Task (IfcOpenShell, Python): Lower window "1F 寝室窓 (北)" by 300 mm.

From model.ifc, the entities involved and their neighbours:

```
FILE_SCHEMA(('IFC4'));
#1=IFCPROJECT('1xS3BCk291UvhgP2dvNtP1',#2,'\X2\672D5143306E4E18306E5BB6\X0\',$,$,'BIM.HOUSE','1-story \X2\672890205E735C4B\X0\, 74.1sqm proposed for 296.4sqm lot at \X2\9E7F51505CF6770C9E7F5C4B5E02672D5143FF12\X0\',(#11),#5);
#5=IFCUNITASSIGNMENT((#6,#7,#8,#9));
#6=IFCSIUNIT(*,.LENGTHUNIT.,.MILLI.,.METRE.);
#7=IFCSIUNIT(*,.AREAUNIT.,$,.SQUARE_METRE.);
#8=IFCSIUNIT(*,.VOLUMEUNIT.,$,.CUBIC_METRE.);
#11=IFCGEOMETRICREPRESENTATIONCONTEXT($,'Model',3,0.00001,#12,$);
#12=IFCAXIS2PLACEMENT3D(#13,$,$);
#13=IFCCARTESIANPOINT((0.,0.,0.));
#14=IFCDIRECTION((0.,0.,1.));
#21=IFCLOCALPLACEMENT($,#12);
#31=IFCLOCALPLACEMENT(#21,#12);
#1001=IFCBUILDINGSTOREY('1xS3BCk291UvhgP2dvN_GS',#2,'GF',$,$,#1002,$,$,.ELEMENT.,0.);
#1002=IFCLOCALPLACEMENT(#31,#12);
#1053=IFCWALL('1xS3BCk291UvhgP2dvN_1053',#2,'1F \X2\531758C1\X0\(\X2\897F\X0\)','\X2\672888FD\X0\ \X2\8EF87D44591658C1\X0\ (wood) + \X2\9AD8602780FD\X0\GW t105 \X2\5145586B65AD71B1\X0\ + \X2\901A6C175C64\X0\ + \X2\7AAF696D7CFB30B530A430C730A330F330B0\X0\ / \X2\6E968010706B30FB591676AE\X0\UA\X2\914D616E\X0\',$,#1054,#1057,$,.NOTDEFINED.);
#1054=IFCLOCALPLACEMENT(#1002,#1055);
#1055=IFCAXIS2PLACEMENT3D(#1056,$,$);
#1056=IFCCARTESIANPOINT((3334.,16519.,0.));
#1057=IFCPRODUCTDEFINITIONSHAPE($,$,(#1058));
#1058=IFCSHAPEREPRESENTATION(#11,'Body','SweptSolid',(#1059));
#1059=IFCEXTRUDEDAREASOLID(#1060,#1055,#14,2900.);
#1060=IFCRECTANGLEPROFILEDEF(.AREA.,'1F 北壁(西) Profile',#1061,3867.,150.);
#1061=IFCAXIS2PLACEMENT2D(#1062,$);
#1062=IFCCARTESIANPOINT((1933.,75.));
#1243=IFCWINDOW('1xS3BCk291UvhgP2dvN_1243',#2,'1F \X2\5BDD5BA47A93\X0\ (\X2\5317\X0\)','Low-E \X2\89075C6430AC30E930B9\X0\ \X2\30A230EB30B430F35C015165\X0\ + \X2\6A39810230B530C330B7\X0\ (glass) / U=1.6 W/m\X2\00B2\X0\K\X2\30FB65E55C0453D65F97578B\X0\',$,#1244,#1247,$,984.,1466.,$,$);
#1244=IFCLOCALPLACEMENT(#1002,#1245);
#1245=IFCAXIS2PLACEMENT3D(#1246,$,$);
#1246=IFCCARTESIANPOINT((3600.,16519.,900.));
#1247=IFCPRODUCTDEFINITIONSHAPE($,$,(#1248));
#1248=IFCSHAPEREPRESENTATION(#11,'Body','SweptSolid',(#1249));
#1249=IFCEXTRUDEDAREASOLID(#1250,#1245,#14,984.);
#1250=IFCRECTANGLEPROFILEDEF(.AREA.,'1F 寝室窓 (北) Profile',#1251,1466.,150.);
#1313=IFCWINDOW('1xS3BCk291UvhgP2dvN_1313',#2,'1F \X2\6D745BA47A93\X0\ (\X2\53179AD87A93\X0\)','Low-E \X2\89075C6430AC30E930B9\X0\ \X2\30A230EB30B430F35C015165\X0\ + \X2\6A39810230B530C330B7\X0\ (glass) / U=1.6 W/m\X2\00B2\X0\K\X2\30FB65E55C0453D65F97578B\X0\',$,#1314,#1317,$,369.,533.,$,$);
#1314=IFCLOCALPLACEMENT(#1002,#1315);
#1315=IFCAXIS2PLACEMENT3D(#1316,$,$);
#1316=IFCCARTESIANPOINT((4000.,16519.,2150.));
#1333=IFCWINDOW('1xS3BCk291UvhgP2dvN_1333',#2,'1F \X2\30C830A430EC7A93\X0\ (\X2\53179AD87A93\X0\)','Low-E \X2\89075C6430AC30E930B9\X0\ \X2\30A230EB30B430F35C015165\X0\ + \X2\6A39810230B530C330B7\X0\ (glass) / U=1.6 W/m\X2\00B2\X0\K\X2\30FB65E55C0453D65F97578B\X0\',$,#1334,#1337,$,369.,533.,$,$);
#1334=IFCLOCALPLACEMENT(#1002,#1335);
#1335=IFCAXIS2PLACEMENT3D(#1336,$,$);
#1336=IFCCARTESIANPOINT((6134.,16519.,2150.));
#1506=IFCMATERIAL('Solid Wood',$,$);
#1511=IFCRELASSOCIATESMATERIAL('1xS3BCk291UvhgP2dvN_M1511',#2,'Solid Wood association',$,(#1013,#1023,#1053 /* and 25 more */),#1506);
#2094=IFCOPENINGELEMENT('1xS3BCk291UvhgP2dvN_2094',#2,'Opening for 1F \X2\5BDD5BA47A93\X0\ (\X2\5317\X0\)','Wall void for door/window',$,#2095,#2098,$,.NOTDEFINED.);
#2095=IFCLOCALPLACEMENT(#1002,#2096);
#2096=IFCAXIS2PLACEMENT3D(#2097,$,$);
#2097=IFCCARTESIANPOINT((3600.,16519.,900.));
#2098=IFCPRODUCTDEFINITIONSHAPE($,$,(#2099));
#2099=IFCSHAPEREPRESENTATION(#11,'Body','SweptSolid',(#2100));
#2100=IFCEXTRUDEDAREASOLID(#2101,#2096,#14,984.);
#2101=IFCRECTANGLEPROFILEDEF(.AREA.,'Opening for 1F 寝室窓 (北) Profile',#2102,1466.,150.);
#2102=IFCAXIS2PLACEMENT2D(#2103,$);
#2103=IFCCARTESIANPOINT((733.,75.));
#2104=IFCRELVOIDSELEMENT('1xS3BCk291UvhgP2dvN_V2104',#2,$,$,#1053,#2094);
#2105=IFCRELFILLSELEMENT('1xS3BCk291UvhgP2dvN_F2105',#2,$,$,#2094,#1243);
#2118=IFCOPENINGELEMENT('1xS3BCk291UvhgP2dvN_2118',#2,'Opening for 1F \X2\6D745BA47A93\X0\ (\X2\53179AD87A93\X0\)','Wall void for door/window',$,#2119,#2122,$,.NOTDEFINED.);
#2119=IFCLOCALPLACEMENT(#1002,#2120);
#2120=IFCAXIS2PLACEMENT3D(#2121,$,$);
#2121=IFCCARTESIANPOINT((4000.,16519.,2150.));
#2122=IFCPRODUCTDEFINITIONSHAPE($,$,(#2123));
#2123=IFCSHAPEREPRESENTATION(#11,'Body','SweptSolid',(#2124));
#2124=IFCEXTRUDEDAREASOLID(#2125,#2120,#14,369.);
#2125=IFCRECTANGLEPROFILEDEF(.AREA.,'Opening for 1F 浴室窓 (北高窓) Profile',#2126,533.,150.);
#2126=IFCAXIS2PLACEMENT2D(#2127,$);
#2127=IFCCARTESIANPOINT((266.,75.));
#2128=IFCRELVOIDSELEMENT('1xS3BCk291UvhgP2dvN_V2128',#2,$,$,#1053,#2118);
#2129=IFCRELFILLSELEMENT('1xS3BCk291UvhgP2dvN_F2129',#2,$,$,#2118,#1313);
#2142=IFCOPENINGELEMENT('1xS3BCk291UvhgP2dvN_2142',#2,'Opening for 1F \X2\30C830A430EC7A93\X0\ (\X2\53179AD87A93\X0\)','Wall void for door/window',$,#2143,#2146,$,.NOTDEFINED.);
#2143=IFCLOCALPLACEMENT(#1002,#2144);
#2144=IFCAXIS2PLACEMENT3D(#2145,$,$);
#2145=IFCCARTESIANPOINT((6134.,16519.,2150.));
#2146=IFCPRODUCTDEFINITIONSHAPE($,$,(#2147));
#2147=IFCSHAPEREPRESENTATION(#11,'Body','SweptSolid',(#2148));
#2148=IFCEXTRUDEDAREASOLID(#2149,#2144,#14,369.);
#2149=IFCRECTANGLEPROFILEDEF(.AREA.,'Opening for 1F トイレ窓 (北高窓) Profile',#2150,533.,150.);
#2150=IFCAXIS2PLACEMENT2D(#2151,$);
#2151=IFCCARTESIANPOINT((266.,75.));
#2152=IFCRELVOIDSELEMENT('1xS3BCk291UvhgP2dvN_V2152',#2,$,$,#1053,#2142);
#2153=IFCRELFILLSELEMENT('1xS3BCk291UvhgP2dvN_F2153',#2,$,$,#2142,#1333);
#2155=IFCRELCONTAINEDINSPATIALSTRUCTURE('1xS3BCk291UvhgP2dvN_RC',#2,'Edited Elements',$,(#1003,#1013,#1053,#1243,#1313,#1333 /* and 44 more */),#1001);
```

```python
import numpy as np
import ifcopenshell
import ifcopenshell.api.geometry
import ifcopenshell.util.placement
import ifcopenshell.util.unit

model = ifcopenshell.open("model.ifc")
unit_scale = ifcopenshell.util.unit.calculate_unit_scale(model)

window = model.by_guid("1xS3BCk291UvhgP2dvN_1243")
opening = window.FillsVoids[0].RelatingOpeningElement
dz = -0.3 / unit_scale

shift = np.array([0.0, 0.0, dz])
# The window is not placed relative to its opening, so move both.
for product in (opening, window):
    matrix = ifcopenshell.util.placement.get_local_placement(product.ObjectPlacement)
    matrix[:3, 3] += shift
    ifcopenshell.api.geometry.edit_object_placement(model, product=product, matrix=matrix, is_si=False)

print(f"moved by {dz * unit_scale:+.3f} m")

model.write("model_updated.ifc")
```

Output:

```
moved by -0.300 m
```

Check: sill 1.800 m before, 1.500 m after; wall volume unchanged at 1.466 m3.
